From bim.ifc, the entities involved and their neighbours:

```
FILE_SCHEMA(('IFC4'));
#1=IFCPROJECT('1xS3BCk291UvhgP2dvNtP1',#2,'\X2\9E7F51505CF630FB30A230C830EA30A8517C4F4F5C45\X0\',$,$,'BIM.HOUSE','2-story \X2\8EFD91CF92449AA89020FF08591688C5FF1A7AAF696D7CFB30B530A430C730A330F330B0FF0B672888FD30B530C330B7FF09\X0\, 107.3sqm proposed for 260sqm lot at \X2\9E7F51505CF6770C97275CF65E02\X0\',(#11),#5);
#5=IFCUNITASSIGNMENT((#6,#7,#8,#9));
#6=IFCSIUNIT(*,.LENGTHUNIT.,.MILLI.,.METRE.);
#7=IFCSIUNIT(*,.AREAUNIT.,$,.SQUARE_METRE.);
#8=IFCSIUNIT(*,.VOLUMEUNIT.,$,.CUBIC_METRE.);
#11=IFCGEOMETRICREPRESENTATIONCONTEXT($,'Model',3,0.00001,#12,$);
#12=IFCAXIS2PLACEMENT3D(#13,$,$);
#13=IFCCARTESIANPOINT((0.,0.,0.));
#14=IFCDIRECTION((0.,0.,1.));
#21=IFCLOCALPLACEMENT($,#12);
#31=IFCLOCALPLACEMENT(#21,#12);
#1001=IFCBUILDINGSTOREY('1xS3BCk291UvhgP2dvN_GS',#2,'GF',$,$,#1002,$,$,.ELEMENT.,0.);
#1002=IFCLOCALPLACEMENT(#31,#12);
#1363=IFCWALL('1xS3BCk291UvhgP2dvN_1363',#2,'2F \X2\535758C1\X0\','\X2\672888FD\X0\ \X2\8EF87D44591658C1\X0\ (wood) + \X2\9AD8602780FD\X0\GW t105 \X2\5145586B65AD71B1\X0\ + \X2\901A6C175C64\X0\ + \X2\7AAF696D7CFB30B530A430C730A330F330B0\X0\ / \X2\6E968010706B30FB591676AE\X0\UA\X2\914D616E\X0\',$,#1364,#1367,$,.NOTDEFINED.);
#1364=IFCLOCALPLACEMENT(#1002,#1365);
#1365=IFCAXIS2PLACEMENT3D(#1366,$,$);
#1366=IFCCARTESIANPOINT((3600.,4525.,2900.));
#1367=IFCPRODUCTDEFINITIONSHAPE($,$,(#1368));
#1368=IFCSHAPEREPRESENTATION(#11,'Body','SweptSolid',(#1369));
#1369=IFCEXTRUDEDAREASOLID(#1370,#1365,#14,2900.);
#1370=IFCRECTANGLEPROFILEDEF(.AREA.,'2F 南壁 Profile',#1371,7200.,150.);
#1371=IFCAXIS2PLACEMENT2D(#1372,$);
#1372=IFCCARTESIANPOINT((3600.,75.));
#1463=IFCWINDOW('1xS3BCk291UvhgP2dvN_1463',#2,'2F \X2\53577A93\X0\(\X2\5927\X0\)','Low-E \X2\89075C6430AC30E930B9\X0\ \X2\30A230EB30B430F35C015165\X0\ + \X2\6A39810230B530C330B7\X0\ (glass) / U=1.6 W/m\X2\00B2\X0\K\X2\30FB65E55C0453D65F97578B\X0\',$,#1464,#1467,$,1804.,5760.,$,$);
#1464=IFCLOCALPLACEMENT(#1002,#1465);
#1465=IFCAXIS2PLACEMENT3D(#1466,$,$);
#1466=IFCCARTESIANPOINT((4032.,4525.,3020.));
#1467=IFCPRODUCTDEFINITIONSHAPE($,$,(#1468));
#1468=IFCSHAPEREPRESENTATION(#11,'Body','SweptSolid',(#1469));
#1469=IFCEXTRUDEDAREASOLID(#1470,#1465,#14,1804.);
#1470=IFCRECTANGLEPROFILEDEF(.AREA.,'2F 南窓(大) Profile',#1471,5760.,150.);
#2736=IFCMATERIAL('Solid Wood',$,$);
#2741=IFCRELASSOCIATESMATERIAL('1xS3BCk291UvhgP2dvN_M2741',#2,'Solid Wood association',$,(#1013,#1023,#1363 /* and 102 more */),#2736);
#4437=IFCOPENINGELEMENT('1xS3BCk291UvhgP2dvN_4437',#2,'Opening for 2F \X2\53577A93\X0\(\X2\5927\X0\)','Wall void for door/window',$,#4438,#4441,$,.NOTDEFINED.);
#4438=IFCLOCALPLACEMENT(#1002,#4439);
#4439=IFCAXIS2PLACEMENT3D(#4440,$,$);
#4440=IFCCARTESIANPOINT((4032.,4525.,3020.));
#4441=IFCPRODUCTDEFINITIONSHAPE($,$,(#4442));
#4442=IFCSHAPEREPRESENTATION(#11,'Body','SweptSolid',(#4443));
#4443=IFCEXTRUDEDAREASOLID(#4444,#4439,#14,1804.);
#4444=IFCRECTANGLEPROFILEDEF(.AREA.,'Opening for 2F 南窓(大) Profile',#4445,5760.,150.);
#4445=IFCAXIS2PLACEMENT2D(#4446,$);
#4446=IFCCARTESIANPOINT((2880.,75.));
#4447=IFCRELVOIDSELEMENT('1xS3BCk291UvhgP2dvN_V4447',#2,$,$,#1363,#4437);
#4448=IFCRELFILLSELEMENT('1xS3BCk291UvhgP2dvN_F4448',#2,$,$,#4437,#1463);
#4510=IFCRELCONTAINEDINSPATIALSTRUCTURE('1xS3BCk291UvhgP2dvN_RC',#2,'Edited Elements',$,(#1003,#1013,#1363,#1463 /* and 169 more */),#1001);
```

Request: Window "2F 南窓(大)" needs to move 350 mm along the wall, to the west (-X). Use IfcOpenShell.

```python
import ifcopenshell
import ifcopenshell.api.geometry
import ifcopenshell.util.placement
import ifcopenshell.util.unit

model = ifcopenshell.open("bim.ifc")
unit_scale = ifcopenshell.util.unit.calculate_unit_scale(model)

window = model.by_id(1463)
opening = window.FillsVoids[0].RelatingOpeningElement
wall = opening.VoidsElements[0].RelatingBuildingElement

wall_matrix = ifcopenshell.util.placement.get_local_placement(wall.ObjectPlacement)
shift = wall_matrix[:3, 0] * -0.35 / unit_scale
before = ifcopenshell.util.placement.get_local_placement(window.ObjectPlacement)[:3, 3].copy()

# The window is not placed relative to its opening, so move both.
for product in (opening, window):
    matrix = ifcopenshell.util.placement.get_local_placement(product.ObjectPlacement)
    matrix[:3, 3] += shift
    ifcopenshell.api.geometry.edit_object_placement(model, product=product, matrix=matrix, is_si=False)

after = ifcopenshell.util.placement.get_local_placement(window.ObjectPlacement)[:3, 3]
print("window moved by", (after - before).round(3) + 0.0)

model.write("bim_rev.ifc")
```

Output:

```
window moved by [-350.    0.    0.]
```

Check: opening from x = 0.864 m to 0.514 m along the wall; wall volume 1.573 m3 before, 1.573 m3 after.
